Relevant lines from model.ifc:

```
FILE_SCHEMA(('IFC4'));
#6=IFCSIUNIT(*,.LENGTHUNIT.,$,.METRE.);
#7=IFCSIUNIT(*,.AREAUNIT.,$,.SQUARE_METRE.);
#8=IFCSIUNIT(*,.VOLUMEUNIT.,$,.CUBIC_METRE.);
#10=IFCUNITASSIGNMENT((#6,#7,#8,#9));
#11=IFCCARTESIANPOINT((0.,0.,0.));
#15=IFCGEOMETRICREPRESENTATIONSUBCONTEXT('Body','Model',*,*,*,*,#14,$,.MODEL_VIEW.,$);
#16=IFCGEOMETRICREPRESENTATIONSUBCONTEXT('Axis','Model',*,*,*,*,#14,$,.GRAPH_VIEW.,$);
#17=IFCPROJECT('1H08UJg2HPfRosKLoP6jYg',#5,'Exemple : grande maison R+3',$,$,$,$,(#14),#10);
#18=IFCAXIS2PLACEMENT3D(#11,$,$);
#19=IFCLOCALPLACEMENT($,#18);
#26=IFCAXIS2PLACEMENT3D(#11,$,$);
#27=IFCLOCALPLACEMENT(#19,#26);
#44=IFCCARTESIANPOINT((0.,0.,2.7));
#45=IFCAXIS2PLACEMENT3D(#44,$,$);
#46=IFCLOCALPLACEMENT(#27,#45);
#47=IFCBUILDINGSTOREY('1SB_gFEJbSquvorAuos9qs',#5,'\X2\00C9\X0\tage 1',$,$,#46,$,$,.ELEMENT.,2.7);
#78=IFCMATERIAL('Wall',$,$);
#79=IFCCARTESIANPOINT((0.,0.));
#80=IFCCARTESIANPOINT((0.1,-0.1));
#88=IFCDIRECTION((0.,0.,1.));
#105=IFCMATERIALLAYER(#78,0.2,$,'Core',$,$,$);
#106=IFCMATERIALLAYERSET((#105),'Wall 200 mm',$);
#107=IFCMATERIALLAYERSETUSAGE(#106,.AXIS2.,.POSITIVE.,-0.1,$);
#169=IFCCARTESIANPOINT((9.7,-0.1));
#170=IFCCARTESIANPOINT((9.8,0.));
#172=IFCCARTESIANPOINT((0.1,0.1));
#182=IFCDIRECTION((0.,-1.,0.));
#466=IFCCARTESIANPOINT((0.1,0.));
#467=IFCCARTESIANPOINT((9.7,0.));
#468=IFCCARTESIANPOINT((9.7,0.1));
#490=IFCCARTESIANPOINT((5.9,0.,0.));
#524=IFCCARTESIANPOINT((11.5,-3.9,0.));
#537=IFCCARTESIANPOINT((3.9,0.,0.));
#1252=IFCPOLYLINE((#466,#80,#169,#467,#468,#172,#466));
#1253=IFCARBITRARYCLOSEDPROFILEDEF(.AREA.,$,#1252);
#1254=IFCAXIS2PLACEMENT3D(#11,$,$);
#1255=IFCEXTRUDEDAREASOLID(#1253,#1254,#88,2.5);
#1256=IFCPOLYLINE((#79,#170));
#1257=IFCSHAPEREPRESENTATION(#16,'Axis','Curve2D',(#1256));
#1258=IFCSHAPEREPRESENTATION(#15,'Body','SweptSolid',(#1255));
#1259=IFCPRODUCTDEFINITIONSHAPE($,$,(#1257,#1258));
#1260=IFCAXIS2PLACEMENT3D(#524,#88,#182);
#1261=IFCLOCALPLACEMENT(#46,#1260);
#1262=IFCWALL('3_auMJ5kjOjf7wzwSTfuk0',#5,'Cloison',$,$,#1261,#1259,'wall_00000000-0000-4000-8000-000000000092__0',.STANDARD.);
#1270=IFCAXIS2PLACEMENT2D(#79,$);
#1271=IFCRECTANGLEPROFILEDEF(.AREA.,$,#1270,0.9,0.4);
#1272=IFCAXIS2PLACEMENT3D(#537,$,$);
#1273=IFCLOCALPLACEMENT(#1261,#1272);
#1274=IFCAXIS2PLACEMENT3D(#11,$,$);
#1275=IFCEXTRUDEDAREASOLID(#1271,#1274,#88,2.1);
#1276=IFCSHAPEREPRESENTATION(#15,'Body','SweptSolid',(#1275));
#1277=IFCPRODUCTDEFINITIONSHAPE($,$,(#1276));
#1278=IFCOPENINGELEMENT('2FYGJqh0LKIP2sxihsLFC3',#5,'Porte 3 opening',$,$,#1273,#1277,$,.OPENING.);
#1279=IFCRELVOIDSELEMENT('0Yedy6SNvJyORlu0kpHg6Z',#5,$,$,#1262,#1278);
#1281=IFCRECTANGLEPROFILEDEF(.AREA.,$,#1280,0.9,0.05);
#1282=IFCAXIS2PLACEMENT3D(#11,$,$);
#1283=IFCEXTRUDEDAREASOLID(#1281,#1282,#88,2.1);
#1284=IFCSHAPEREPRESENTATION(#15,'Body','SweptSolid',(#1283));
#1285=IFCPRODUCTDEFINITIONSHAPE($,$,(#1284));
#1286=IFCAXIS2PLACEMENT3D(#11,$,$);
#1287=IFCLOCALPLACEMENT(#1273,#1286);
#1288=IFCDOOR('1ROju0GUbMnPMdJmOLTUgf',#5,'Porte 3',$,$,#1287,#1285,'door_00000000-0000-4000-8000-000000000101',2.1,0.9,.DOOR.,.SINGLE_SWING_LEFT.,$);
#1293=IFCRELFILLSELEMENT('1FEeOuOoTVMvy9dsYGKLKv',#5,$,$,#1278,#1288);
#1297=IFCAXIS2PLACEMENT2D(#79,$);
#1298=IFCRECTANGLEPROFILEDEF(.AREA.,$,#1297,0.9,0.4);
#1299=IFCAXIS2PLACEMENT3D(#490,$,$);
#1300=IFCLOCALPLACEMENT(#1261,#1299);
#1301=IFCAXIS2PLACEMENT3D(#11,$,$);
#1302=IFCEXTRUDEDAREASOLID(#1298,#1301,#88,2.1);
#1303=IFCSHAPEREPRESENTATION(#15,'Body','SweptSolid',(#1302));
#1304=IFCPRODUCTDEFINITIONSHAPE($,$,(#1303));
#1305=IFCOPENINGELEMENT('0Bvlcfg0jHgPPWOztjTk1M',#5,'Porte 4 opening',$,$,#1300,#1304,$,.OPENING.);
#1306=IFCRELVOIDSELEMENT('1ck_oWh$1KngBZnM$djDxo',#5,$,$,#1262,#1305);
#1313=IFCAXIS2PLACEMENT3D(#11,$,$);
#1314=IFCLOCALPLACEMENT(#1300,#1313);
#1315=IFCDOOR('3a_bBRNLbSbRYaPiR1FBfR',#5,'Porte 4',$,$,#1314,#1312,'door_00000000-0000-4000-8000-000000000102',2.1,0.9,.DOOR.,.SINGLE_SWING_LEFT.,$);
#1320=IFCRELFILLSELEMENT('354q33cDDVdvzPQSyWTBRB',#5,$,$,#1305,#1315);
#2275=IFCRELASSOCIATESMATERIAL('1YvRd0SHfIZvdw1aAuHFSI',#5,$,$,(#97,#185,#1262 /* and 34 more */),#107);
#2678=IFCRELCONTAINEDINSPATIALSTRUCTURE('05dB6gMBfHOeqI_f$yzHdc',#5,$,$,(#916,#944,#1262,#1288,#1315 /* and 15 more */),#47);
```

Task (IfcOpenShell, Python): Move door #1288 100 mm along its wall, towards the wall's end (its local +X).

```python
import ifcopenshell
import ifcopenshell.api.geometry
import ifcopenshell.util.placement
import ifcopenshell.util.unit

model = ifcopenshell.open("model.ifc")
unit_scale = ifcopenshell.util.unit.calculate_unit_scale(model)

door = model.by_guid("1ROju0GUbMnPMdJmOLTUgf")
opening = door.FillsVoids[0].RelatingOpeningElement
wall = opening.VoidsElements[0].RelatingBuildingElement

wall_matrix = ifcopenshell.util.placement.get_local_placement(wall.ObjectPlacement)
shift = wall_matrix[:3, 0] * 0.1 / unit_scale
before = ifcopenshell.util.placement.get_local_placement(door.ObjectPlacement)[:3, 3].copy()

# The door is placed relative to its opening, so it follows when the opening moves.
matrix = ifcopenshell.util.placement.get_local_placement(opening.ObjectPlacement)
matrix[:3, 3] += shift
ifcopenshell.api.geometry.edit_object_placement(
    model, product=opening, matrix=matrix, is_si=False, should_transform_children=True
)

after = ifcopenshell.util.placement.get_local_placement(door.ObjectPlacement)[:3, 3]
print("door moved by", (after - before).round(3) + 0.0)

model.write("model_updated.ifc")
```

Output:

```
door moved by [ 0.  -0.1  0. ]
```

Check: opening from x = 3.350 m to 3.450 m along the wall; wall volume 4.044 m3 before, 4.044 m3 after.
